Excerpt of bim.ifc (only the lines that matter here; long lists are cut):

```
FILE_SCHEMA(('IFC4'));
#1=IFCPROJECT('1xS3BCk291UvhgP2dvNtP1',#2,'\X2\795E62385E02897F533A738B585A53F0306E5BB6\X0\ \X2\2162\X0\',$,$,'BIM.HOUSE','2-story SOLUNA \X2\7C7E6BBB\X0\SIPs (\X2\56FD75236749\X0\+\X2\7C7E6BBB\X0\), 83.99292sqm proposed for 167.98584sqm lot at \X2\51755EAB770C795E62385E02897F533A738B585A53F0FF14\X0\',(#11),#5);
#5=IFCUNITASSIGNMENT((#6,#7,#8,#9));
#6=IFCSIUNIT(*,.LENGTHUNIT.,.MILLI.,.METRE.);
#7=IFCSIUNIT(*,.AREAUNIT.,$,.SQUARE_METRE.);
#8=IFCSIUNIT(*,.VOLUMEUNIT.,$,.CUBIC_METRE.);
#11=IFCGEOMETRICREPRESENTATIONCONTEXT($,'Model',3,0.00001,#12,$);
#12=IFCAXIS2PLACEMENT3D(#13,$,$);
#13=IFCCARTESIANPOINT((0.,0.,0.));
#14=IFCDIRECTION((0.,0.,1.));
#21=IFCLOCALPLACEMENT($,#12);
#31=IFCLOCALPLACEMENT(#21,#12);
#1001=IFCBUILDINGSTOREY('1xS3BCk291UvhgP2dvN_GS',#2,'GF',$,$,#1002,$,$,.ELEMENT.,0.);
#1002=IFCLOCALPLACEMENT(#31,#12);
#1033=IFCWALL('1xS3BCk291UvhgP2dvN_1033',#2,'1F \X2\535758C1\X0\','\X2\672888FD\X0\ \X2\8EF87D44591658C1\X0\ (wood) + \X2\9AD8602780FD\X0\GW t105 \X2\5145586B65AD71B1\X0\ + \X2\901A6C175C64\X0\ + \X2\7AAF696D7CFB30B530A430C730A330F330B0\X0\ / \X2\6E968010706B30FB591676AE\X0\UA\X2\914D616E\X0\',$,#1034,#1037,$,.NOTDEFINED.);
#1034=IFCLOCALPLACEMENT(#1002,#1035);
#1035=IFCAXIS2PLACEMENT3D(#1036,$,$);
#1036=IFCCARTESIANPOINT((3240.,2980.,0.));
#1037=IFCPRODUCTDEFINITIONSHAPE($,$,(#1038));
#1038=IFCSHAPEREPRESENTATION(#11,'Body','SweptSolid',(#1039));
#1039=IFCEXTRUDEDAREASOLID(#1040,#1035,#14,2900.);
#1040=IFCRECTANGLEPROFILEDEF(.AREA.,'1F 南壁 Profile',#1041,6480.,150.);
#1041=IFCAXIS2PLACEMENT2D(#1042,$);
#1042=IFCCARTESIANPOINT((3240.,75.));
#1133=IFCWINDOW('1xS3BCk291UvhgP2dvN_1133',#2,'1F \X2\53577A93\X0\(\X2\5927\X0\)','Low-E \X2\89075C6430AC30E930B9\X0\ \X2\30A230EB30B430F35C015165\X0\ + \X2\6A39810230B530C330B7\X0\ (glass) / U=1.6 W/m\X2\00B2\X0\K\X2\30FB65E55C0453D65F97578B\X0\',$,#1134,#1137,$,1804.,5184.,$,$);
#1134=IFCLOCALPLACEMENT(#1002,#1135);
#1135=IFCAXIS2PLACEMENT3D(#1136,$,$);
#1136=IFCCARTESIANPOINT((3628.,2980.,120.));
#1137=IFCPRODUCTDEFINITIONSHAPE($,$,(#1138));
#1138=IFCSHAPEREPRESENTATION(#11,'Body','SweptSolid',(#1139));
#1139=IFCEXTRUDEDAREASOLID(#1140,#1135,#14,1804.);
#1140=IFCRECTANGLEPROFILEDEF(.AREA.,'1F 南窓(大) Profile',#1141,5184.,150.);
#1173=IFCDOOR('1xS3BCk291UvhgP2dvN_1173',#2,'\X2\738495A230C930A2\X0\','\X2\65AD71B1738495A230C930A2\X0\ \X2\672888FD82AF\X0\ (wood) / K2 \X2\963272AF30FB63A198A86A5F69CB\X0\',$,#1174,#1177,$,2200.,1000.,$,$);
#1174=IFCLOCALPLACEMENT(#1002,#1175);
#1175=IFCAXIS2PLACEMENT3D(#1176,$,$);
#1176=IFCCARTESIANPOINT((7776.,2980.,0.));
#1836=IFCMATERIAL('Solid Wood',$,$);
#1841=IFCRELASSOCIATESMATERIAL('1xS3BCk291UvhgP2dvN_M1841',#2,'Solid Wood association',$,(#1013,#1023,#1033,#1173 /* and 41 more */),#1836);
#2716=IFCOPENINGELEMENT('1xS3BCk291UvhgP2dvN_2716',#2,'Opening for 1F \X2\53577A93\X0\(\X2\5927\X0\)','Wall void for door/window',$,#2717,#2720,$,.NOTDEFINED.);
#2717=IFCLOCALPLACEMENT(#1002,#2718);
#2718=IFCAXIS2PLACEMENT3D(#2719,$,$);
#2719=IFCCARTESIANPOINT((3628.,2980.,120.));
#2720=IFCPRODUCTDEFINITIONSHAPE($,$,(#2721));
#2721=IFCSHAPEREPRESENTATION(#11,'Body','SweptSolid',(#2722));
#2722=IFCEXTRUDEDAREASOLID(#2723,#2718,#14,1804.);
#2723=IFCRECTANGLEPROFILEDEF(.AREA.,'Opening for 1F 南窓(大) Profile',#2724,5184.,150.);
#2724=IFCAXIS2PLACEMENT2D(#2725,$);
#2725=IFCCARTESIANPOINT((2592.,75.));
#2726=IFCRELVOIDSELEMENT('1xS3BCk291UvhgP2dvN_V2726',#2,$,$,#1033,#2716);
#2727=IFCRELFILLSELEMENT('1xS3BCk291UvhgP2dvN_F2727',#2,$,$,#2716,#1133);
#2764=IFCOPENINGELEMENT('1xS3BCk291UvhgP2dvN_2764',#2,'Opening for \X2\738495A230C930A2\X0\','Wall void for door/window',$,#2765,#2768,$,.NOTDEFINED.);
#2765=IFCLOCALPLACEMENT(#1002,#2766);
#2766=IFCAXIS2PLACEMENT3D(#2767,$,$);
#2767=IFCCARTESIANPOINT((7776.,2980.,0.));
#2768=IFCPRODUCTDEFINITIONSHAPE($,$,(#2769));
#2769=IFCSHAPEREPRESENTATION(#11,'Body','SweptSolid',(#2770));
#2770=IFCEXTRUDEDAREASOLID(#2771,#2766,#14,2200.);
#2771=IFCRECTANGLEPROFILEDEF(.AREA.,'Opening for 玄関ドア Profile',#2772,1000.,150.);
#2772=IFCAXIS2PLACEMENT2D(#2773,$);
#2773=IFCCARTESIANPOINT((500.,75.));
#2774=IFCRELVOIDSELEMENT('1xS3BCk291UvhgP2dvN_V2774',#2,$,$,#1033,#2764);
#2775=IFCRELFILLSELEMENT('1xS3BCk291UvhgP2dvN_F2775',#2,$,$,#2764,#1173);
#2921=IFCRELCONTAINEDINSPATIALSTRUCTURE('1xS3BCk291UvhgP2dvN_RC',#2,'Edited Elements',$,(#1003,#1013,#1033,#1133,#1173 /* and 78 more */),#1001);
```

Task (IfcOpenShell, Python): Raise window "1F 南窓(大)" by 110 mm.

```python
import numpy as np
import ifcopenshell
import ifcopenshell.api.geometry
import ifcopenshell.util.placement
import ifcopenshell.util.unit

model = ifcopenshell.open("bim.ifc")
unit_scale = ifcopenshell.util.unit.calculate_unit_scale(model)

window = model.by_guid("1xS3BCk291UvhgP2dvN_1133")
opening = window.FillsVoids[0].RelatingOpeningElement
dz = 0.11 / unit_scale

shift = np.array([0.0, 0.0, dz])
# The window is not placed relative to its opening, so move both.
for product in (opening, window):
    matrix = ifcopenshell.util.placement.get_local_placement(product.ObjectPlacement)
    matrix[:3, 3] += shift
    ifcopenshell.api.geometry.edit_object_placement(model, product=product, matrix=matrix, is_si=False)

print(f"moved by {dz * unit_scale:+.3f} m")

model.write("bim_rev.ifc")
```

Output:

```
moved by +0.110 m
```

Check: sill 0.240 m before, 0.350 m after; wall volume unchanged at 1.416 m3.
